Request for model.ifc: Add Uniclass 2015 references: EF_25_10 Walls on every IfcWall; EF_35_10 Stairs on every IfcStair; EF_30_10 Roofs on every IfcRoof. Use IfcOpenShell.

First a look at what the model holds.

```python
import ifcopenshell

model = ifcopenshell.open("model.ifc")
print(model.schema)
print("classifications:", [c.Name for c in model.by_type("IfcClassification")])
for ifc_class in ("IfcDoor", "IfcRoof", "IfcStair", "IfcWall", "IfcWindow"):
    print(ifc_class, len(model.by_type(ifc_class)))
```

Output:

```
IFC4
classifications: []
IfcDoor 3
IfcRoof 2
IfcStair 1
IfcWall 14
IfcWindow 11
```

```python
import ifcopenshell
import ifcopenshell.api.classification

model = ifcopenshell.open("model.ifc")

system = ifcopenshell.api.classification.add_classification(model, classification="Uniclass 2015")

codes = {
    "IfcWall": ("EF_25_10", "Walls"),
    "IfcStair": ("EF_35_10", "Stairs"),
    "IfcRoof": ("EF_30_10", "Roofs"),
}
for ifc_class, (code, name) in codes.items():
    products = model.by_type(ifc_class)
    ifcopenshell.api.classification.add_reference(
        model, products=products, classification=system, identification=code, name=name
    )
    print(code, len(products))

model.write("model-out.ifc")
```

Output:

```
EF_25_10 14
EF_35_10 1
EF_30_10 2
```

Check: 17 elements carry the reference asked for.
